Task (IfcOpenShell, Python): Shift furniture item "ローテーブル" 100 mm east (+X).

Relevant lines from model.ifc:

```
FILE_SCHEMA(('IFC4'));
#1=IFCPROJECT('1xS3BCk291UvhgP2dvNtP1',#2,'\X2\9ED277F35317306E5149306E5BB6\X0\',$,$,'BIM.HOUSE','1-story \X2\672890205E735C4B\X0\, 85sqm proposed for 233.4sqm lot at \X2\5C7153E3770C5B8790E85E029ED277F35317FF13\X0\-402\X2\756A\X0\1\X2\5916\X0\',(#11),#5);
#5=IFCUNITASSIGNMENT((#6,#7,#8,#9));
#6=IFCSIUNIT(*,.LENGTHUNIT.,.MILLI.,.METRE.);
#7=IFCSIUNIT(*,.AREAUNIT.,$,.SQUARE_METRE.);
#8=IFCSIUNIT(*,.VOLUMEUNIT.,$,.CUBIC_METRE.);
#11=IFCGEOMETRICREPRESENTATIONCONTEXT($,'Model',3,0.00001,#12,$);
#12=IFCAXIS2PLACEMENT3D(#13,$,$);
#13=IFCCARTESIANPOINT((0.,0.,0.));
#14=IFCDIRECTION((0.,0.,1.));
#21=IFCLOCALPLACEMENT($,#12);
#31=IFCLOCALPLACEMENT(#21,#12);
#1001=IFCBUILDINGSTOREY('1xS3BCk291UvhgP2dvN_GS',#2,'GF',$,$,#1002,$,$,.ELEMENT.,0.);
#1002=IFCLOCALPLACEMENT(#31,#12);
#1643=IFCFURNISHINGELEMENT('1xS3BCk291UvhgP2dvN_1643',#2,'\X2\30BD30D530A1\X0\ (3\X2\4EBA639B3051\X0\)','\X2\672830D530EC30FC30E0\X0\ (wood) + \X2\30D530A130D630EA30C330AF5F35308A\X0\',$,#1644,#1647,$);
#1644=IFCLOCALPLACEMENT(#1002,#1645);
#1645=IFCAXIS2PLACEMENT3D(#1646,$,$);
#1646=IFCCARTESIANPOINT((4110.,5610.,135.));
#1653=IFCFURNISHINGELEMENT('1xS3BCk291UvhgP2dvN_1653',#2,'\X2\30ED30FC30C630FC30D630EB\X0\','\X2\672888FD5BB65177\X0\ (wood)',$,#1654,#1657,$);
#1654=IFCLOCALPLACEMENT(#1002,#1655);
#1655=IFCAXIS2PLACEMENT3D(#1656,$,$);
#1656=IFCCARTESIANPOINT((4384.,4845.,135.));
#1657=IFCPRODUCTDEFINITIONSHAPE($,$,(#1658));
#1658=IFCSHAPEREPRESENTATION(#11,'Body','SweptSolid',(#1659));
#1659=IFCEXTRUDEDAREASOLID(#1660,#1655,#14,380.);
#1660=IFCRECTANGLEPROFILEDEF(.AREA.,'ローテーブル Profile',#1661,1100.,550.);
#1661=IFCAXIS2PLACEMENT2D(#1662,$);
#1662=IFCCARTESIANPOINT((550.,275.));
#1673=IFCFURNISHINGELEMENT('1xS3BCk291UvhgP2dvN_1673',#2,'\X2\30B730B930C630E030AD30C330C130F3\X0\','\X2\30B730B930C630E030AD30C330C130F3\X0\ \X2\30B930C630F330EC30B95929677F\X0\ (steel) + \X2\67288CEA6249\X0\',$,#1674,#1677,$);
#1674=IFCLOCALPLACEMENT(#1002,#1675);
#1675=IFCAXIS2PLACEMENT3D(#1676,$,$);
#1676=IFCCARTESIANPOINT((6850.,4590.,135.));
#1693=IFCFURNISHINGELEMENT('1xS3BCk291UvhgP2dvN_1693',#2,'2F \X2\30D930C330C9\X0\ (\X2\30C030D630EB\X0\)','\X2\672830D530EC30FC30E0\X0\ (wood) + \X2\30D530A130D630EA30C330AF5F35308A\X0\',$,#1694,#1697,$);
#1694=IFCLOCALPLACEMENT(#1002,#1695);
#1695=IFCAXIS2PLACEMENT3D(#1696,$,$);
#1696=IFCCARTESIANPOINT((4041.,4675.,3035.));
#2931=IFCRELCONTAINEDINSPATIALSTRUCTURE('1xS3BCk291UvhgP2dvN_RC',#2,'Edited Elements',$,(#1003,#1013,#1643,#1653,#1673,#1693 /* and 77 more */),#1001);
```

```python
import ifcopenshell
import ifcopenshell.api.geometry
import ifcopenshell.util.placement

model = ifcopenshell.open("model.ifc")

item = model.by_id(1653)
matrix = ifcopenshell.util.placement.get_local_placement(item.ObjectPlacement)
matrix[0, 3] += 100.0
ifcopenshell.api.geometry.edit_object_placement(model, product=item, matrix=matrix, is_si=False)

print(ifcopenshell.util.placement.get_local_placement(item.ObjectPlacement).round(3) + 0.0)

model.write("model_rev.ifc")
```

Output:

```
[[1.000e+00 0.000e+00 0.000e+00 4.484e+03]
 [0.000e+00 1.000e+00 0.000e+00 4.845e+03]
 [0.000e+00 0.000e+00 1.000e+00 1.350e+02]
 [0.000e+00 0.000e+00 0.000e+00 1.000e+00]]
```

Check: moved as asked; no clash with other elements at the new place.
